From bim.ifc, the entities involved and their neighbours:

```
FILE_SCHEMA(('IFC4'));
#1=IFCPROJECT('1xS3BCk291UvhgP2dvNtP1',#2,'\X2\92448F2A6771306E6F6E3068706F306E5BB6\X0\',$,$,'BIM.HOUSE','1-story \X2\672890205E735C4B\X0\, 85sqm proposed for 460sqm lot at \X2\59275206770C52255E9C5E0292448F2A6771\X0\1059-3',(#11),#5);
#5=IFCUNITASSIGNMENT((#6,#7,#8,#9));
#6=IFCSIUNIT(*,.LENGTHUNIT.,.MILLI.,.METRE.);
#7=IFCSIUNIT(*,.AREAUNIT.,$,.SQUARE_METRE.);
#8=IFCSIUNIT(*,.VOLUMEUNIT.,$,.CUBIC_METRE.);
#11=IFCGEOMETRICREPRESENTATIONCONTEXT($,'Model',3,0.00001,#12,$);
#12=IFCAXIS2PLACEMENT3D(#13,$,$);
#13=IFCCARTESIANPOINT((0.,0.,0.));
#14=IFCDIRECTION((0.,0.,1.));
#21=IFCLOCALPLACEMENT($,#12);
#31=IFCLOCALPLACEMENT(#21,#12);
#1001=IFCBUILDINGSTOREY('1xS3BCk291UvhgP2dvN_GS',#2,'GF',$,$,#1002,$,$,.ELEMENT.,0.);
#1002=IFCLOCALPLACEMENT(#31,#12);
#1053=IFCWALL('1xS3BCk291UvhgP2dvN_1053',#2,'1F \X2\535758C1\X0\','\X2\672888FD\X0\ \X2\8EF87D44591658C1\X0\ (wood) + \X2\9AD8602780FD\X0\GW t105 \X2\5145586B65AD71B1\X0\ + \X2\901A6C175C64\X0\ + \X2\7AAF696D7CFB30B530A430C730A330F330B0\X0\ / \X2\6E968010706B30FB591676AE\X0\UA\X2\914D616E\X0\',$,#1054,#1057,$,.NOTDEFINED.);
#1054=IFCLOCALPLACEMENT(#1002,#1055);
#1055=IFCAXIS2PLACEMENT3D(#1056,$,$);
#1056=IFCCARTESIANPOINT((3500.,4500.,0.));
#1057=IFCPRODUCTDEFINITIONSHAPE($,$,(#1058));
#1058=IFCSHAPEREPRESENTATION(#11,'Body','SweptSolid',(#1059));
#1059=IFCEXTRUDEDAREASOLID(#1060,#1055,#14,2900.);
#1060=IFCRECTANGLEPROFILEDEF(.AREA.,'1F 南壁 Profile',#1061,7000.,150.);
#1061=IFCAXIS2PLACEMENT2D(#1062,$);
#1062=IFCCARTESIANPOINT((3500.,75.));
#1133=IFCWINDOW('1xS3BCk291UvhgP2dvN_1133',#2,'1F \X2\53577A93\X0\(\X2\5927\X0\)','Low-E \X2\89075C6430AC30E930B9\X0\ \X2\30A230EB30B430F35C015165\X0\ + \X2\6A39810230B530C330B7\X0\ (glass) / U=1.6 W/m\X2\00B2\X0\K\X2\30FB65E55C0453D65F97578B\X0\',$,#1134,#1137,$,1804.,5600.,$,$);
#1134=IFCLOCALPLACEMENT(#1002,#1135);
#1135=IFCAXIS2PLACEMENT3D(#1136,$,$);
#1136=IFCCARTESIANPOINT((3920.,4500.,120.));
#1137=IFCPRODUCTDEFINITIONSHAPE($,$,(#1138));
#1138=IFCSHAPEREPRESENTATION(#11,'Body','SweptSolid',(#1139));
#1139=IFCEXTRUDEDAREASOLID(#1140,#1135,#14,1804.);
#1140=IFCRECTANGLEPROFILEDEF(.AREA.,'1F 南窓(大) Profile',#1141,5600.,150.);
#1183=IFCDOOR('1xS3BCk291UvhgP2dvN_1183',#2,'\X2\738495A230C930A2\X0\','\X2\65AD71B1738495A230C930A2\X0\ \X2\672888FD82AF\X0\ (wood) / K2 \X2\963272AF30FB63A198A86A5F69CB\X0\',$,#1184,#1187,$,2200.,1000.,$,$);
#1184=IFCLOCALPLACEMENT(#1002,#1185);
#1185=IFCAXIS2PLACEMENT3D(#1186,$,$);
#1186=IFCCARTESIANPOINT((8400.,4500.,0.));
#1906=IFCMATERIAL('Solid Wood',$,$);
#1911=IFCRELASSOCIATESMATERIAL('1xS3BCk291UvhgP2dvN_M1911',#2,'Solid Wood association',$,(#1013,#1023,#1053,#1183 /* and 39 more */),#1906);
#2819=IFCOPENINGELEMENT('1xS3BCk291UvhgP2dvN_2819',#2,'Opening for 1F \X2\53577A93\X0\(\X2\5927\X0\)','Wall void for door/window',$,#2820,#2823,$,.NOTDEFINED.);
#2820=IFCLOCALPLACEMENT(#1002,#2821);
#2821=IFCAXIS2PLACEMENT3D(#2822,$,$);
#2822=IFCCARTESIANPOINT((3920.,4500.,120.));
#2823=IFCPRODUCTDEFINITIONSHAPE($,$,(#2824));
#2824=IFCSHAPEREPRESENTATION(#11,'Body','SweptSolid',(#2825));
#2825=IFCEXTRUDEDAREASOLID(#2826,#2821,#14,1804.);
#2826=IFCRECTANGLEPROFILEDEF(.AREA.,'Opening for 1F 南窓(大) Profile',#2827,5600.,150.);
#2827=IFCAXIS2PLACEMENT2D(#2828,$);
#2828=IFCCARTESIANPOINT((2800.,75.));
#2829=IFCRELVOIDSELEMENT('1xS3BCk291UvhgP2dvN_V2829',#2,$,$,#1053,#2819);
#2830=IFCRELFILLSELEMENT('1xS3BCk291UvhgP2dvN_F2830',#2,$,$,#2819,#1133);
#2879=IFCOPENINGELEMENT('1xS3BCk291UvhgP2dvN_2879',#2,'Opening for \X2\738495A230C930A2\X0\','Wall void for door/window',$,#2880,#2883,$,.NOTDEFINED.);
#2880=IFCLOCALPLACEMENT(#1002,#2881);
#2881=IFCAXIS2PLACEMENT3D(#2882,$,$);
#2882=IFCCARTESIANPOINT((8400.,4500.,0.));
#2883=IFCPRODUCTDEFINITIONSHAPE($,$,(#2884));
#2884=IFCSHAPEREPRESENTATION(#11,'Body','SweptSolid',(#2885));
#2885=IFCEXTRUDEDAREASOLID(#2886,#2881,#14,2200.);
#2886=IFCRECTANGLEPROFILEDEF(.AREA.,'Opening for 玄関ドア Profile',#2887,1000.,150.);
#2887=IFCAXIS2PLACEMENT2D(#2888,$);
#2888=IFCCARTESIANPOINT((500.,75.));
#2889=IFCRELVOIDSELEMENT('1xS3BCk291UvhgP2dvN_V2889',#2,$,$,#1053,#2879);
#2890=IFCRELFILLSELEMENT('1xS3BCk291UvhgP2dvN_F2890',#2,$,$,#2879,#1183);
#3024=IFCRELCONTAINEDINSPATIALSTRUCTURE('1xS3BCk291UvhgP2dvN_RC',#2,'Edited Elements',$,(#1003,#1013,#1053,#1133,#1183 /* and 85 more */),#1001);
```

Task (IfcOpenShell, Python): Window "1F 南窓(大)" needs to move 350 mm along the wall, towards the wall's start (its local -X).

```python
import ifcopenshell
import ifcopenshell.api.geometry
import ifcopenshell.util.placement
import ifcopenshell.util.unit

model = ifcopenshell.open("bim.ifc")
unit_scale = ifcopenshell.util.unit.calculate_unit_scale(model)

window = model.by_guid("1xS3BCk291UvhgP2dvN_1133")
opening = window.FillsVoids[0].RelatingOpeningElement
wall = opening.VoidsElements[0].RelatingBuildingElement

wall_matrix = ifcopenshell.util.placement.get_local_placement(wall.ObjectPlacement)
shift = wall_matrix[:3, 0] * -0.35 / unit_scale
before = ifcopenshell.util.placement.get_local_placement(window.ObjectPlacement)[:3, 3].copy()

# The window is not placed relative to its opening, so move both.
for product in (opening, window):
    matrix = ifcopenshell.util.placement.get_local_placement(product.ObjectPlacement)
    matrix[:3, 3] += shift
    ifcopenshell.api.geometry.edit_object_placement(model, product=product, matrix=matrix, is_si=False)

after = ifcopenshell.util.placement.get_local_placement(window.ObjectPlacement)[:3, 3]
print("window moved by", (after - before).round(3) + 0.0)

model.write("bim_edited.ifc")
```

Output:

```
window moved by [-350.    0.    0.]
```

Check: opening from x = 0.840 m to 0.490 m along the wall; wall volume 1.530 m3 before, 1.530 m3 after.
